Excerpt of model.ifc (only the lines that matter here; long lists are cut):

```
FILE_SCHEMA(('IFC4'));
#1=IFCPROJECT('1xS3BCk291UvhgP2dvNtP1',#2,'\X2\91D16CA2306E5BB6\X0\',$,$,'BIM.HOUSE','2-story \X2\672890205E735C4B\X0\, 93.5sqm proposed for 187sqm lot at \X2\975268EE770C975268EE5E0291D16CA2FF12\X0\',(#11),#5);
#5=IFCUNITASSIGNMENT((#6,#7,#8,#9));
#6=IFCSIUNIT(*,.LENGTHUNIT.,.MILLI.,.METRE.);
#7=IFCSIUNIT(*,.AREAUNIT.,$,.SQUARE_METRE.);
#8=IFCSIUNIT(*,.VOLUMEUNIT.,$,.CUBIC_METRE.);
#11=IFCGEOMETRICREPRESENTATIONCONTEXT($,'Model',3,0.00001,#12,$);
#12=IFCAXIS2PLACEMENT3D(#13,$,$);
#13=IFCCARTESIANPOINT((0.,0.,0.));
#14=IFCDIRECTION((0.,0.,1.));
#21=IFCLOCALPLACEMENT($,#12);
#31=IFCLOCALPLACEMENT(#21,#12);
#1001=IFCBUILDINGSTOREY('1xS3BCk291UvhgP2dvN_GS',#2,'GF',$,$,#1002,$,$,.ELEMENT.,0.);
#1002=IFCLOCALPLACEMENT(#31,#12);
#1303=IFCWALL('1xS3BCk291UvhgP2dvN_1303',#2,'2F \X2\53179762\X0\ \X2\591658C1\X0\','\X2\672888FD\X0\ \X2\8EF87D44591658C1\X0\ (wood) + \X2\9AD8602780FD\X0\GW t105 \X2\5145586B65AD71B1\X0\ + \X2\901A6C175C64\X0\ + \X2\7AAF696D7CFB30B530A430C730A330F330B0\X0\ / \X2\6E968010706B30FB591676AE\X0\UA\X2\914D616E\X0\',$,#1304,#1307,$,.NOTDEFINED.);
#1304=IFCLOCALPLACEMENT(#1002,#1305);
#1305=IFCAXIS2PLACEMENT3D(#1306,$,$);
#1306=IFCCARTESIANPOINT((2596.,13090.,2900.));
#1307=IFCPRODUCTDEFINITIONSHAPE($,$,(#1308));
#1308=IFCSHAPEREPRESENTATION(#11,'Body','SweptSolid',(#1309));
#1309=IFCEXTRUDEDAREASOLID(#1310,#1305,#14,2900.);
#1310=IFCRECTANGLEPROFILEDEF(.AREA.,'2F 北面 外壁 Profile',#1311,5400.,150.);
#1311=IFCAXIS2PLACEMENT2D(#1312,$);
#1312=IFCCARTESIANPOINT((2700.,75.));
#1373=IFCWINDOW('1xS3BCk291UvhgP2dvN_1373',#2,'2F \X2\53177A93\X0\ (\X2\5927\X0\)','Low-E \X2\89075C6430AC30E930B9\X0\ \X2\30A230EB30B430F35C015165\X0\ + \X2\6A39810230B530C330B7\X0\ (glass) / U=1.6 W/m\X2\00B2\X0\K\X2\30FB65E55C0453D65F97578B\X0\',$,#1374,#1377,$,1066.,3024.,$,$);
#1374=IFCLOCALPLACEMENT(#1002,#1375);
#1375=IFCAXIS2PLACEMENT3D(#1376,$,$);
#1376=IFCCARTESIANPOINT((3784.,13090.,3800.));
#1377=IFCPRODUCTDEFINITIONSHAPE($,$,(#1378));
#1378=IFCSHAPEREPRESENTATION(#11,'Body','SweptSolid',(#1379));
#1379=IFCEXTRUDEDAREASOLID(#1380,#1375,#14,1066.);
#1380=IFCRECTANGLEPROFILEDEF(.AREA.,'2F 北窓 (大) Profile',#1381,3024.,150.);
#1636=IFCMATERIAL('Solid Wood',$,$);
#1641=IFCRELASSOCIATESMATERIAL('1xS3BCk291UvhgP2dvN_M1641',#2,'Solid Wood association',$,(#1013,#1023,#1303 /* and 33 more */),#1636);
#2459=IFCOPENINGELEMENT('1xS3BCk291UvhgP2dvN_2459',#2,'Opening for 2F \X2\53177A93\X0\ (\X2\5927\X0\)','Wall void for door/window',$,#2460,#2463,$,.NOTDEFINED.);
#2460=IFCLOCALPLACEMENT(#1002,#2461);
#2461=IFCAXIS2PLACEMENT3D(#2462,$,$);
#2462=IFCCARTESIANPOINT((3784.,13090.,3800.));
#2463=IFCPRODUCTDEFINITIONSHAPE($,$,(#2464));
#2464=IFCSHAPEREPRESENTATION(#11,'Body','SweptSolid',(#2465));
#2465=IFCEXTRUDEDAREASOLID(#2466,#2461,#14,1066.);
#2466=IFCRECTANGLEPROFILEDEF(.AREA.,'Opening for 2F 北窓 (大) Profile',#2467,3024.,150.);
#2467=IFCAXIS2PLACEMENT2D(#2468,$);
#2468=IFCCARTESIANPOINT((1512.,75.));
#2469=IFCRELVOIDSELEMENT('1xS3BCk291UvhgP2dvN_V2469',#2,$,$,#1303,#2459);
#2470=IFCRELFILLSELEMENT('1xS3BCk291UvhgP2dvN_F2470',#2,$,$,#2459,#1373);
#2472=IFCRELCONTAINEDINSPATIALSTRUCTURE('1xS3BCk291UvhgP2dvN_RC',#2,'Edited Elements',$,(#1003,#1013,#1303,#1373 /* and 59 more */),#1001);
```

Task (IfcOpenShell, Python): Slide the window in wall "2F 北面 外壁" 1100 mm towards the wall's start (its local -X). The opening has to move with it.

```python
import ifcopenshell
import ifcopenshell.api.geometry
import ifcopenshell.util.placement
import ifcopenshell.util.unit

model = ifcopenshell.open("model.ifc")
unit_scale = ifcopenshell.util.unit.calculate_unit_scale(model)

window = model.by_id(1373)
opening = window.FillsVoids[0].RelatingOpeningElement
wall = opening.VoidsElements[0].RelatingBuildingElement

wall_matrix = ifcopenshell.util.placement.get_local_placement(wall.ObjectPlacement)
shift = wall_matrix[:3, 0] * -1.1 / unit_scale
before = ifcopenshell.util.placement.get_local_placement(window.ObjectPlacement)[:3, 3].copy()

# The window is not placed relative to its opening, so move both.
for product in (opening, window):
    matrix = ifcopenshell.util.placement.get_local_placement(product.ObjectPlacement)
    matrix[:3, 3] += shift
    ifcopenshell.api.geometry.edit_object_placement(model, product=product, matrix=matrix, is_si=False)

after = ifcopenshell.util.placement.get_local_placement(window.ObjectPlacement)[:3, 3]
print("window moved by", (after - before).round(3) + 0.0)

model.write("model_edited.ifc")
```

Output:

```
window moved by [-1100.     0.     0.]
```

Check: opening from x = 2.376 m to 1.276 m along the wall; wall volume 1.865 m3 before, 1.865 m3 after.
